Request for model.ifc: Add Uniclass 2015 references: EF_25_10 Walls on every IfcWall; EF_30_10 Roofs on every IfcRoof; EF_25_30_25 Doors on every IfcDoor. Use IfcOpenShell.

First a look at what the model holds.

```python
import ifcopenshell

model = ifcopenshell.open("model.ifc")
print(model.schema)
print("classifications:", [c.Name for c in model.by_type("IfcClassification")])
for ifc_class in ("IfcDoor", "IfcRoof", "IfcStair", "IfcWall", "IfcWindow"):
    print(ifc_class, len(model.by_type(ifc_class)))
```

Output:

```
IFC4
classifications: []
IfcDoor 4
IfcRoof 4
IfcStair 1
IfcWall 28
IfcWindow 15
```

```python
import ifcopenshell
import ifcopenshell.api.classification

model = ifcopenshell.open("model.ifc")

system = ifcopenshell.api.classification.add_classification(model, classification="Uniclass 2015")

codes = {
    "IfcWall": ("EF_25_10", "Walls"),
    "IfcRoof": ("EF_30_10", "Roofs"),
    "IfcDoor": ("EF_25_30_25", "Doors"),
}
for ifc_class, (code, name) in codes.items():
    products = model.by_type(ifc_class)
    ifcopenshell.api.classification.add_reference(
        model, products=products, classification=system, identification=code, name=name
    )
    print(code, len(products))

model.write("model_updated.ifc")
```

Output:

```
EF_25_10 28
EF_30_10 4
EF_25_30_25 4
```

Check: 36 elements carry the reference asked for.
